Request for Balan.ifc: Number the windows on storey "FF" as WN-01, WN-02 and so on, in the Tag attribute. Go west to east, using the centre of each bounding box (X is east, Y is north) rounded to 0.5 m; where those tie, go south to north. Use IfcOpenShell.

First a look at what the model holds.

```python
import ifcopenshell
import ifcopenshell.util.element
import ifcopenshell.util.placement

model = ifcopenshell.open("Balan.ifc")
print(model.schema)
storey = next(s for s in model.by_type("IfcBuildingStorey") if s.Name == "FF")
windows = [e for e in ifcopenshell.util.element.get_decomposition(storey) if e.is_a("IfcWindow")]
for e in sorted(windows, key=lambda e: e.id()):
    origin = ifcopenshell.util.placement.get_local_placement(e.ObjectPlacement)[:3, 3]
    print(e.id(), e.Tag, e.Name, origin.round(2) + 0.0, sep=" | ")
```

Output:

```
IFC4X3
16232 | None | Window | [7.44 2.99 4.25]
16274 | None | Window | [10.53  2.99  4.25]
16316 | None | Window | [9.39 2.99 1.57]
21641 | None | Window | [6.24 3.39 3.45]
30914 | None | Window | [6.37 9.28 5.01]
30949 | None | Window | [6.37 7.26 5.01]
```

```python
import ifcopenshell
import ifcopenshell.geom
import ifcopenshell.util.element
import ifcopenshell.util.shape

model = ifcopenshell.open("Balan.ifc")
settings = ifcopenshell.geom.settings()
settings.set("use-world-coords", True)


def centre(element):
    shape = ifcopenshell.geom.create_shape(settings, element)
    return ifcopenshell.util.shape.get_bbox_centroid(shape.geometry)


storey = next(s for s in model.by_type("IfcBuildingStorey") if s.Name == "FF")
windows = [e for e in ifcopenshell.util.element.get_decomposition(storey) if e.is_a("IfcWindow")]

# Insertion points can sit at a corner or the storey origin, so sort by the geometry (in metres).
centres = {e: centre(e) for e in windows}
windows.sort(key=lambda e: (round(centres[e][0] / 0.5), centres[e][1]))

for i, e in enumerate(windows, start=1):
    number = f"WN-{i:02d}"
    e.Tag = number
    print(e.id(), number)

model.write("Balan_v2.ifc")
```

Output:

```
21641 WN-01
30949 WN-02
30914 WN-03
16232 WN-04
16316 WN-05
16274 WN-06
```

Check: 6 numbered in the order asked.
